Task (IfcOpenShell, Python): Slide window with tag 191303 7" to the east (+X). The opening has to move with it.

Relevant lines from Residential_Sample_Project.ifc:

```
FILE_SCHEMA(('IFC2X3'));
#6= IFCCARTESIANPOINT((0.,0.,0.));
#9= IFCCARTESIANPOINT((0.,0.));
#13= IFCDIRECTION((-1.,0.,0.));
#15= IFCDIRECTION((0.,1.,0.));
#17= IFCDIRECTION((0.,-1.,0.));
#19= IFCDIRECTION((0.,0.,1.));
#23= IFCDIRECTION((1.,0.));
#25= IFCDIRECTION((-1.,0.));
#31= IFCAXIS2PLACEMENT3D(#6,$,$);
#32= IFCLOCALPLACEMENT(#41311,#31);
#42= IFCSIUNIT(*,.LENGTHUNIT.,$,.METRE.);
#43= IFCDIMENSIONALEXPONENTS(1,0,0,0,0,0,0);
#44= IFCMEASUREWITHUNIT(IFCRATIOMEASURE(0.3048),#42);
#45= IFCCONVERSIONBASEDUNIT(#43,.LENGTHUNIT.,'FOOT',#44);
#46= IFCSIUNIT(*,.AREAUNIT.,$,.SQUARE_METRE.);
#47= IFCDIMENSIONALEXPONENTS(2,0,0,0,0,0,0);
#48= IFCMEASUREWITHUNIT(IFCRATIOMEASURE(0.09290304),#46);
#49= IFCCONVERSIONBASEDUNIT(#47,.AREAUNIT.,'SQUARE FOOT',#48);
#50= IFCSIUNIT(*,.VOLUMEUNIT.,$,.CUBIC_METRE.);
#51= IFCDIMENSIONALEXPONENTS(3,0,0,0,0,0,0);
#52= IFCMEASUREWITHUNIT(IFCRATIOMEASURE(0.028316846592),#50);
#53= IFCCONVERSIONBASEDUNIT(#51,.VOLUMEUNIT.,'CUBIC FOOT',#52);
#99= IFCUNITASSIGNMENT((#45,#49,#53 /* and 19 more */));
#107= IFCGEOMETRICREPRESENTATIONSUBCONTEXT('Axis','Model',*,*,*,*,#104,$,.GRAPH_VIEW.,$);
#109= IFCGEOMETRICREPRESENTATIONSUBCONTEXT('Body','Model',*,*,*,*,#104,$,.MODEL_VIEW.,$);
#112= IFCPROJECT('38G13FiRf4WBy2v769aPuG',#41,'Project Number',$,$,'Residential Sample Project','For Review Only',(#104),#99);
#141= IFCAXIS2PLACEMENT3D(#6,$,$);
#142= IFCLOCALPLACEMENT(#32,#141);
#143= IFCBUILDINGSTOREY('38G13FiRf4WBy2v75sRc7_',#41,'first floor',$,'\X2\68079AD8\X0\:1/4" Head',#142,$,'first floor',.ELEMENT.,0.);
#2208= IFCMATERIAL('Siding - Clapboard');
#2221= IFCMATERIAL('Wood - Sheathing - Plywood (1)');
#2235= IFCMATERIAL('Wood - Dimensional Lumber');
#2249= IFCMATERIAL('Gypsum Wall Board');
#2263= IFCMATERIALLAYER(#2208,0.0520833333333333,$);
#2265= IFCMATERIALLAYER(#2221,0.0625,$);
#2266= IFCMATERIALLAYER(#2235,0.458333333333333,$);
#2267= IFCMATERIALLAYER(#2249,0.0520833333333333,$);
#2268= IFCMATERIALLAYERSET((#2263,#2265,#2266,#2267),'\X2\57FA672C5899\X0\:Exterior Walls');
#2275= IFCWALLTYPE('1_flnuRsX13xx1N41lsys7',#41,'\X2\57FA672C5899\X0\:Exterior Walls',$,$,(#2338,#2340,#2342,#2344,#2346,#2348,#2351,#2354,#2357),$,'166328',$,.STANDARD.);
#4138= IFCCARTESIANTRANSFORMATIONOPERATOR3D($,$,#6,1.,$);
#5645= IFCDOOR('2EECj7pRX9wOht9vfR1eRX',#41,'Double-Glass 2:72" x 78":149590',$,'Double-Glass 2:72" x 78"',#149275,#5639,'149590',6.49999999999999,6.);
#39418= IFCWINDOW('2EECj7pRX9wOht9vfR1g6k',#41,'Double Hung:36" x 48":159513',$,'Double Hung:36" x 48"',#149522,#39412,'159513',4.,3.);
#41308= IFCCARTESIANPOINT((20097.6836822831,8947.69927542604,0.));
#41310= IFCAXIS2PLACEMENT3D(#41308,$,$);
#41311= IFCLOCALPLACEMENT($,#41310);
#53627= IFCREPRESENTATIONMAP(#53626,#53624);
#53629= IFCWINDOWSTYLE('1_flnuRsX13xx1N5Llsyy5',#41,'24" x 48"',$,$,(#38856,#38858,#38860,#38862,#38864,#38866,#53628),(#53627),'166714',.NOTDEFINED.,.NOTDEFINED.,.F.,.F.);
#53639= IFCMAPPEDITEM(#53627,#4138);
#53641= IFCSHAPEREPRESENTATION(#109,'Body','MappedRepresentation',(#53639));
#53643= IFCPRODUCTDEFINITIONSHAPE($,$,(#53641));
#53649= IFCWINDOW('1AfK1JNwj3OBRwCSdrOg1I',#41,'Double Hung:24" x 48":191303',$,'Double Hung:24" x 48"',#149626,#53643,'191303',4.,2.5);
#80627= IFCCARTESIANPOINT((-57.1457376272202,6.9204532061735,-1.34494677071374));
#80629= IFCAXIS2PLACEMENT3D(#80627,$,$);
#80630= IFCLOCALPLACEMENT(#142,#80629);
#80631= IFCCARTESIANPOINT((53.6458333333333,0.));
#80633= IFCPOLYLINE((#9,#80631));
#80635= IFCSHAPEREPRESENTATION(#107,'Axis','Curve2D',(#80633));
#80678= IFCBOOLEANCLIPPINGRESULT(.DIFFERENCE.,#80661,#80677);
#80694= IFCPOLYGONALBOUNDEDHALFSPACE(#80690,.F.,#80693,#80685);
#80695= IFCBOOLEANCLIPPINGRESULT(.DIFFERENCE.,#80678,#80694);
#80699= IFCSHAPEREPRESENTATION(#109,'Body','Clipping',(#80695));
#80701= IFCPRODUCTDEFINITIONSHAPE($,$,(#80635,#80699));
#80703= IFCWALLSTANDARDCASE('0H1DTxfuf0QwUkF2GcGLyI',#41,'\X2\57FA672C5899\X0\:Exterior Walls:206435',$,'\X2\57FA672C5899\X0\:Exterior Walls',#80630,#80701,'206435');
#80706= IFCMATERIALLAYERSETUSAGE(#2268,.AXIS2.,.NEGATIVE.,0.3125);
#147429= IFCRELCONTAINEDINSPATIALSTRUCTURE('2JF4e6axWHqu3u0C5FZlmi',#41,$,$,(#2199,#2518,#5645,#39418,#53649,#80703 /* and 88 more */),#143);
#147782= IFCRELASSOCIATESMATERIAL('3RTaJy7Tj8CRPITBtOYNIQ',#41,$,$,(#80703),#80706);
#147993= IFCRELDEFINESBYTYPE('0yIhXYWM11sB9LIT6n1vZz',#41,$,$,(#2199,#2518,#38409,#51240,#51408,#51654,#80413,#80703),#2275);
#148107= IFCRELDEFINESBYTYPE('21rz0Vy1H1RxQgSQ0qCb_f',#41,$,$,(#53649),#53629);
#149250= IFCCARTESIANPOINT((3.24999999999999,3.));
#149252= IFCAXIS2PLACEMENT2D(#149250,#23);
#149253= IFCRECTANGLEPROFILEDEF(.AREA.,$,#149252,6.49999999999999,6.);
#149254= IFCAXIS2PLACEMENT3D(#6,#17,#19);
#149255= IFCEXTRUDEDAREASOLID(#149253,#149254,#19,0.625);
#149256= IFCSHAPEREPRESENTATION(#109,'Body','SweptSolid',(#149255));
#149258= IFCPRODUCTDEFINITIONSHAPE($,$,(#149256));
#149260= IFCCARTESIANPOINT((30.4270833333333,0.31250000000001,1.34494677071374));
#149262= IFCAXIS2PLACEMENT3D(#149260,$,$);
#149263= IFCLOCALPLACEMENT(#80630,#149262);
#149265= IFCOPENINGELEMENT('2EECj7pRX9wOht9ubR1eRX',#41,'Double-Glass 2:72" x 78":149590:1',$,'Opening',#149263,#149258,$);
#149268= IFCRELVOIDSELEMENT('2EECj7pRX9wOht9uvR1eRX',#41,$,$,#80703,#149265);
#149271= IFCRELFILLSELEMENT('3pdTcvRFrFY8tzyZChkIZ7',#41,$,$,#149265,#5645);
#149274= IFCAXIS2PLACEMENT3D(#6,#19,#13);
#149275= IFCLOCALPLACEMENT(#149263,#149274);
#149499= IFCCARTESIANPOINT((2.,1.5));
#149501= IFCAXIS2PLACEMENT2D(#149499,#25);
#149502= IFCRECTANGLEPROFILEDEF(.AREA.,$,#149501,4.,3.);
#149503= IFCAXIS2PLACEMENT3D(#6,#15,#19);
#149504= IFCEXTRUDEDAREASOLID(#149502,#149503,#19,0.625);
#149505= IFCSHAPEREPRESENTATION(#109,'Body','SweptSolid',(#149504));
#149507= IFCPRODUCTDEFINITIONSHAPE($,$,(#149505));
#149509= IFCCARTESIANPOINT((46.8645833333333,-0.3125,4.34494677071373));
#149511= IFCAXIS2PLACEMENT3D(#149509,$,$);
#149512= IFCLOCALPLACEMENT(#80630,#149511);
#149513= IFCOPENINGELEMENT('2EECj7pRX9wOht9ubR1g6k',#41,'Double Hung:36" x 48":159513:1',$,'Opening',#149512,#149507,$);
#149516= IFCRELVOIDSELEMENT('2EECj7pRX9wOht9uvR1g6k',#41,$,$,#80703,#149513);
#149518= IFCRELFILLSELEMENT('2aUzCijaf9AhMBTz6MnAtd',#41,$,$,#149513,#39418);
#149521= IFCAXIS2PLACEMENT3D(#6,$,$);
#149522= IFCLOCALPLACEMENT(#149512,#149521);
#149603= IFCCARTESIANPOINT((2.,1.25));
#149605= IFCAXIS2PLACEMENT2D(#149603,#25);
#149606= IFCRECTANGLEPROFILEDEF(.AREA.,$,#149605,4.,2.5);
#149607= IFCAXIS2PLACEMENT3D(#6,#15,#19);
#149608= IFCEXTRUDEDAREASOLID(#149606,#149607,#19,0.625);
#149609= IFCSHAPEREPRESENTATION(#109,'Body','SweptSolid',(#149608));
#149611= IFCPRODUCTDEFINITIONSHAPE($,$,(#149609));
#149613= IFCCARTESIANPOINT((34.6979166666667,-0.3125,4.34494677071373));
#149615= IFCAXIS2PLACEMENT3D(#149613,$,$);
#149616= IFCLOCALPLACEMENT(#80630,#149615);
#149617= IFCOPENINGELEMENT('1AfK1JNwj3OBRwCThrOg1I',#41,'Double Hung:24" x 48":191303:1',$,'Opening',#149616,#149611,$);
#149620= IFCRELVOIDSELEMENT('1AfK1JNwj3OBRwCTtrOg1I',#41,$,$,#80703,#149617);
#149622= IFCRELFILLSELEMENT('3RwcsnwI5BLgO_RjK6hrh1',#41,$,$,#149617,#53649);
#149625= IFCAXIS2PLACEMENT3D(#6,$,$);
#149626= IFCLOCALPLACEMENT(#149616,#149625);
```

```python
import ifcopenshell
import ifcopenshell.api.geometry
import ifcopenshell.util.placement
import ifcopenshell.util.unit

model = ifcopenshell.open("Residential_Sample_Project.ifc")
unit_scale = ifcopenshell.util.unit.calculate_unit_scale(model)

window = model.by_guid("1AfK1JNwj3OBRwCSdrOg1I")
opening = window.FillsVoids[0].RelatingOpeningElement
wall = opening.VoidsElements[0].RelatingBuildingElement

wall_matrix = ifcopenshell.util.placement.get_local_placement(wall.ObjectPlacement)
shift = wall_matrix[:3, 0] * 7 * 0.0254 / unit_scale
before = ifcopenshell.util.placement.get_local_placement(window.ObjectPlacement)[:3, 3].copy()

# The window is placed relative to its opening, so it follows when the opening moves.
matrix = ifcopenshell.util.placement.get_local_placement(opening.ObjectPlacement)
matrix[:3, 3] += shift
ifcopenshell.api.geometry.edit_object_placement(
    model, product=opening, matrix=matrix, is_si=False, should_transform_children=True
)

after = ifcopenshell.util.placement.get_local_placement(window.ObjectPlacement)[:3, 3]
print("window moved by", (after - before).round(3) + 0.0)

model.write("Residential_Sample_Project_updated.ifc")
```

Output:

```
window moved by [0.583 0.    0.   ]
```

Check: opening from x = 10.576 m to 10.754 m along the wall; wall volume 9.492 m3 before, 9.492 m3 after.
